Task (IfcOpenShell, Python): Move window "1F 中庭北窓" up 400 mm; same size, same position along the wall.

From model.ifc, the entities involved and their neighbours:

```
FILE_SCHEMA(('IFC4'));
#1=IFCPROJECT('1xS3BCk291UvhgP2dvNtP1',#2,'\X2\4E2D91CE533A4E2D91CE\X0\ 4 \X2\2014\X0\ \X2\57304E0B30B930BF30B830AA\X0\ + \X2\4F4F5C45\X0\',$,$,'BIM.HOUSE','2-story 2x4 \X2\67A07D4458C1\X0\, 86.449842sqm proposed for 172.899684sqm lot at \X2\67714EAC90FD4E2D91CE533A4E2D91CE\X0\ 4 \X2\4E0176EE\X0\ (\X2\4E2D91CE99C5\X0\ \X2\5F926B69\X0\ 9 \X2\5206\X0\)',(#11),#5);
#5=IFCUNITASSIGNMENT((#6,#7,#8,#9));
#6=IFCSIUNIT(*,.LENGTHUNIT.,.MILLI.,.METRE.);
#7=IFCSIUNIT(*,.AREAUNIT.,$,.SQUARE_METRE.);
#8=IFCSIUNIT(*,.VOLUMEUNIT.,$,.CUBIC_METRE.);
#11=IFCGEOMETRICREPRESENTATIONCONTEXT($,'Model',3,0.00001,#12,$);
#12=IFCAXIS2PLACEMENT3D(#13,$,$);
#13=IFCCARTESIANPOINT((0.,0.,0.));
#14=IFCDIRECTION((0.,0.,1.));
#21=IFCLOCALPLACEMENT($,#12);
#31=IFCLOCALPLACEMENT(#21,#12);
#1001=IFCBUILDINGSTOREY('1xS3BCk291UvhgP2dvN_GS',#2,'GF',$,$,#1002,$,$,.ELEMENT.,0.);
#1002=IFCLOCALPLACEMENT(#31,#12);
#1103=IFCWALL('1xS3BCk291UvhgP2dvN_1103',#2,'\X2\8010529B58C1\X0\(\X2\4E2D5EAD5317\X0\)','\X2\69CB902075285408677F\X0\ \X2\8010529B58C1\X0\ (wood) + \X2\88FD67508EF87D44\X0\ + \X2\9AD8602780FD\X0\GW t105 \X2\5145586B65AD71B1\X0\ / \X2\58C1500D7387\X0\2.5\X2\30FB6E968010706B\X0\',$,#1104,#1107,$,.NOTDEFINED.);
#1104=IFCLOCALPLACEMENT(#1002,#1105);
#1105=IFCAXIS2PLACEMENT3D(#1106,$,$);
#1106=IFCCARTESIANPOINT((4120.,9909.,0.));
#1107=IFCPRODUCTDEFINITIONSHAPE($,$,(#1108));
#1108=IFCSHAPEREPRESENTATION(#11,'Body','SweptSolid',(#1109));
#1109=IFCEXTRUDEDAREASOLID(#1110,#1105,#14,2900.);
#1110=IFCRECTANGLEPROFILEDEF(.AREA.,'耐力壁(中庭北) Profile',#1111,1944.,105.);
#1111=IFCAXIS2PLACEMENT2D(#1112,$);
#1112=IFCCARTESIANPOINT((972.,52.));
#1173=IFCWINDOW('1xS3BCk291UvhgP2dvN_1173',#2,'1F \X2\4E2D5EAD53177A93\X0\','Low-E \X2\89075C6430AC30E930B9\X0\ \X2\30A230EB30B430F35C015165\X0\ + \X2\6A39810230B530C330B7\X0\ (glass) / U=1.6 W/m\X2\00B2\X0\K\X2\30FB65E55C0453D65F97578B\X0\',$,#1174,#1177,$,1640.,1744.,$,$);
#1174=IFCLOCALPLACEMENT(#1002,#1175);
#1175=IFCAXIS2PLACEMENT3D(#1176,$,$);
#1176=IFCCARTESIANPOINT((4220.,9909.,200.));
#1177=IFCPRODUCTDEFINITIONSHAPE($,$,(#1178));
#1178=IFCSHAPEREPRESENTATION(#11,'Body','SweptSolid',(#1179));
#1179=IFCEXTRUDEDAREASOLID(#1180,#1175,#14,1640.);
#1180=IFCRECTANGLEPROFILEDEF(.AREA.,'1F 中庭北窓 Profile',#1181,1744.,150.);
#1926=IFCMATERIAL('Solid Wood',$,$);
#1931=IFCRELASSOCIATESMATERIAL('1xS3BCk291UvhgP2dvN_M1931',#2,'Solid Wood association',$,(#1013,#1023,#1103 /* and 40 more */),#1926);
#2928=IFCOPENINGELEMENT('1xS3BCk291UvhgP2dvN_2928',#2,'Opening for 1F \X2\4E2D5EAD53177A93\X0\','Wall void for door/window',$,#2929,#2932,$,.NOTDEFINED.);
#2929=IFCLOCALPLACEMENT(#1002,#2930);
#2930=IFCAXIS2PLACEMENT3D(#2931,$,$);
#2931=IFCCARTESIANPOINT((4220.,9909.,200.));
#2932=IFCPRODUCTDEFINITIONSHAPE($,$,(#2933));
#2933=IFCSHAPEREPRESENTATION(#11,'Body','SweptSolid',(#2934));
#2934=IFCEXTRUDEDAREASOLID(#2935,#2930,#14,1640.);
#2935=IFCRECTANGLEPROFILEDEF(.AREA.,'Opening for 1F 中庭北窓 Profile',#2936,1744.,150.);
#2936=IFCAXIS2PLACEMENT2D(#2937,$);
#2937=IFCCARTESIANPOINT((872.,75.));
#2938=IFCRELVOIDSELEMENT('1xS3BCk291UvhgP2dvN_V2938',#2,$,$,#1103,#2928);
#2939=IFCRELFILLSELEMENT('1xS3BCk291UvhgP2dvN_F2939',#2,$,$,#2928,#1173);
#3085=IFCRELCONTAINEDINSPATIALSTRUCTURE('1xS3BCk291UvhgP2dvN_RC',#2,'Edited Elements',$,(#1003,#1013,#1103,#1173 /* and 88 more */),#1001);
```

```python
import numpy as np
import ifcopenshell
import ifcopenshell.api.geometry
import ifcopenshell.util.placement
import ifcopenshell.util.unit

model = ifcopenshell.open("model.ifc")
unit_scale = ifcopenshell.util.unit.calculate_unit_scale(model)

window = model.by_guid("1xS3BCk291UvhgP2dvN_1173")
opening = window.FillsVoids[0].RelatingOpeningElement
dz = 400.0

shift = np.array([0.0, 0.0, dz])
# The window is not placed relative to its opening, so move both.
for product in (opening, window):
    matrix = ifcopenshell.util.placement.get_local_placement(product.ObjectPlacement)
    matrix[:3, 3] += shift
    ifcopenshell.api.geometry.edit_object_placement(model, product=product, matrix=matrix, is_si=False)

print(f"moved by {dz * unit_scale:+.3f} m")

model.write("model-out.ifc")
```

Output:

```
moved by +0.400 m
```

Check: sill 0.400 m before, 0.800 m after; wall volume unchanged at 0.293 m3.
